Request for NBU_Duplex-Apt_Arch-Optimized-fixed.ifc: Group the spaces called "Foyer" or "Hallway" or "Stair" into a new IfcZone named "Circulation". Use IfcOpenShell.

First a look at what the model holds.

```python
import ifcopenshell

model = ifcopenshell.open("NBU_Duplex-Apt_Arch-Optimized-fixed.ifc")
print(model.schema)
seen = {}
for space in model.by_type("IfcSpace"):
    seen[space.LongName] = seen.get(space.LongName, 0) + 1
for name, count in sorted(seen.items(), key=str):
    print(count, "x", name)
print("zones:", [z.Name for z in model.by_type("IfcZone")][:20])
```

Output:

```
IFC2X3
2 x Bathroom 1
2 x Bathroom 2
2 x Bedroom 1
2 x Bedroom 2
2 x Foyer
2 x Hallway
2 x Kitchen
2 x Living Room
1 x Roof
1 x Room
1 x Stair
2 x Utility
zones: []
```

```python
import ifcopenshell
import ifcopenshell.api.group
import ifcopenshell.api.root

model = ifcopenshell.open("NBU_Duplex-Apt_Arch-Optimized-fixed.ifc")

names = {"Foyer", "Hallway", "Stair"}
spaces = [s for s in model.by_type("IfcSpace") if s.LongName in names]

zone = ifcopenshell.api.root.create_entity(model, ifc_class="IfcZone", name="Circulation")
ifcopenshell.api.group.assign_group(model, products=spaces, group=zone)
print(len(spaces), "spaces in", zone.Name)

model.write("NBU_Duplex-Apt_Arch-Optimized-fixed-out.ifc")
```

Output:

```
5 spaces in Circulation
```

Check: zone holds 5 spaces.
